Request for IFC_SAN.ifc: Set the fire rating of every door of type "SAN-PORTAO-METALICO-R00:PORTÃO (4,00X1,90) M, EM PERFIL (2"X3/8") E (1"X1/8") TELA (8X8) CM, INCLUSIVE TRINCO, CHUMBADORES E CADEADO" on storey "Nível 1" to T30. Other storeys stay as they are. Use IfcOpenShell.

First a look at what the model holds.

```python
import ifcopenshell
import ifcopenshell.util.element

model = ifcopenshell.open("IFC_SAN.ifc")
print(model.schema)
storey = next(s for s in model.by_type("IfcBuildingStorey") if s.Name == "Nível 1")
doors = [e for e in ifcopenshell.util.element.get_decomposition(storey) if e.is_a("IfcDoor")]
seen = {}
for e in doors:
    element_type = ifcopenshell.util.element.get_type(e)
    key = (element_type.Name if element_type != e and element_type else None, ifcopenshell.util.element.get_pset(e, "Pset_DoorCommon", "FireRating"))
    seen[key] = seen.get(key, 0) + 1
for (name, value), count in sorted(seen.items(), key=str):
    print(count, "x", name, "|", value)
```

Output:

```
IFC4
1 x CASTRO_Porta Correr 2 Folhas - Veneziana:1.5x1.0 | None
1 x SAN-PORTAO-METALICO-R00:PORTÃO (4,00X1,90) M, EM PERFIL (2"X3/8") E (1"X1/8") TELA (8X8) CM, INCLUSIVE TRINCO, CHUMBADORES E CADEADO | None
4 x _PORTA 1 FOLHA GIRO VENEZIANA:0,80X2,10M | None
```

```python
import ifcopenshell
import ifcopenshell.api.pset
import ifcopenshell.util.element

model = ifcopenshell.open("IFC_SAN.ifc")

storey = next(s for s in model.by_type("IfcBuildingStorey") if s.Name == "Nível 1")
doors = [e for e in ifcopenshell.util.element.get_decomposition(storey) if e.is_a("IfcDoor")]

count = 0
for e in doors:
    element_type = ifcopenshell.util.element.get_type(e)
    if element_type in (None, e) or element_type.Name != 'SAN-PORTAO-METALICO-R00:PORTÃO (4,00X1,90) M, EM PERFIL (2"X3/8") E (1"X1/8") TELA (8X8) CM, INCLUSIVE TRINCO, CHUMBADORES E CADEADO':
        continue
    # add_pset returns the element's existing set when there is one.
    pset = ifcopenshell.api.pset.add_pset(model, product=e, name="Pset_DoorCommon")
    ifcopenshell.api.pset.edit_pset(model, pset=pset, properties={"FireRating": "T30"})
    count += 1

print(count, "doors updated")

model.write("IFC_SAN_updated.ifc")
```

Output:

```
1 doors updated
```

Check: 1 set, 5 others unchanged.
